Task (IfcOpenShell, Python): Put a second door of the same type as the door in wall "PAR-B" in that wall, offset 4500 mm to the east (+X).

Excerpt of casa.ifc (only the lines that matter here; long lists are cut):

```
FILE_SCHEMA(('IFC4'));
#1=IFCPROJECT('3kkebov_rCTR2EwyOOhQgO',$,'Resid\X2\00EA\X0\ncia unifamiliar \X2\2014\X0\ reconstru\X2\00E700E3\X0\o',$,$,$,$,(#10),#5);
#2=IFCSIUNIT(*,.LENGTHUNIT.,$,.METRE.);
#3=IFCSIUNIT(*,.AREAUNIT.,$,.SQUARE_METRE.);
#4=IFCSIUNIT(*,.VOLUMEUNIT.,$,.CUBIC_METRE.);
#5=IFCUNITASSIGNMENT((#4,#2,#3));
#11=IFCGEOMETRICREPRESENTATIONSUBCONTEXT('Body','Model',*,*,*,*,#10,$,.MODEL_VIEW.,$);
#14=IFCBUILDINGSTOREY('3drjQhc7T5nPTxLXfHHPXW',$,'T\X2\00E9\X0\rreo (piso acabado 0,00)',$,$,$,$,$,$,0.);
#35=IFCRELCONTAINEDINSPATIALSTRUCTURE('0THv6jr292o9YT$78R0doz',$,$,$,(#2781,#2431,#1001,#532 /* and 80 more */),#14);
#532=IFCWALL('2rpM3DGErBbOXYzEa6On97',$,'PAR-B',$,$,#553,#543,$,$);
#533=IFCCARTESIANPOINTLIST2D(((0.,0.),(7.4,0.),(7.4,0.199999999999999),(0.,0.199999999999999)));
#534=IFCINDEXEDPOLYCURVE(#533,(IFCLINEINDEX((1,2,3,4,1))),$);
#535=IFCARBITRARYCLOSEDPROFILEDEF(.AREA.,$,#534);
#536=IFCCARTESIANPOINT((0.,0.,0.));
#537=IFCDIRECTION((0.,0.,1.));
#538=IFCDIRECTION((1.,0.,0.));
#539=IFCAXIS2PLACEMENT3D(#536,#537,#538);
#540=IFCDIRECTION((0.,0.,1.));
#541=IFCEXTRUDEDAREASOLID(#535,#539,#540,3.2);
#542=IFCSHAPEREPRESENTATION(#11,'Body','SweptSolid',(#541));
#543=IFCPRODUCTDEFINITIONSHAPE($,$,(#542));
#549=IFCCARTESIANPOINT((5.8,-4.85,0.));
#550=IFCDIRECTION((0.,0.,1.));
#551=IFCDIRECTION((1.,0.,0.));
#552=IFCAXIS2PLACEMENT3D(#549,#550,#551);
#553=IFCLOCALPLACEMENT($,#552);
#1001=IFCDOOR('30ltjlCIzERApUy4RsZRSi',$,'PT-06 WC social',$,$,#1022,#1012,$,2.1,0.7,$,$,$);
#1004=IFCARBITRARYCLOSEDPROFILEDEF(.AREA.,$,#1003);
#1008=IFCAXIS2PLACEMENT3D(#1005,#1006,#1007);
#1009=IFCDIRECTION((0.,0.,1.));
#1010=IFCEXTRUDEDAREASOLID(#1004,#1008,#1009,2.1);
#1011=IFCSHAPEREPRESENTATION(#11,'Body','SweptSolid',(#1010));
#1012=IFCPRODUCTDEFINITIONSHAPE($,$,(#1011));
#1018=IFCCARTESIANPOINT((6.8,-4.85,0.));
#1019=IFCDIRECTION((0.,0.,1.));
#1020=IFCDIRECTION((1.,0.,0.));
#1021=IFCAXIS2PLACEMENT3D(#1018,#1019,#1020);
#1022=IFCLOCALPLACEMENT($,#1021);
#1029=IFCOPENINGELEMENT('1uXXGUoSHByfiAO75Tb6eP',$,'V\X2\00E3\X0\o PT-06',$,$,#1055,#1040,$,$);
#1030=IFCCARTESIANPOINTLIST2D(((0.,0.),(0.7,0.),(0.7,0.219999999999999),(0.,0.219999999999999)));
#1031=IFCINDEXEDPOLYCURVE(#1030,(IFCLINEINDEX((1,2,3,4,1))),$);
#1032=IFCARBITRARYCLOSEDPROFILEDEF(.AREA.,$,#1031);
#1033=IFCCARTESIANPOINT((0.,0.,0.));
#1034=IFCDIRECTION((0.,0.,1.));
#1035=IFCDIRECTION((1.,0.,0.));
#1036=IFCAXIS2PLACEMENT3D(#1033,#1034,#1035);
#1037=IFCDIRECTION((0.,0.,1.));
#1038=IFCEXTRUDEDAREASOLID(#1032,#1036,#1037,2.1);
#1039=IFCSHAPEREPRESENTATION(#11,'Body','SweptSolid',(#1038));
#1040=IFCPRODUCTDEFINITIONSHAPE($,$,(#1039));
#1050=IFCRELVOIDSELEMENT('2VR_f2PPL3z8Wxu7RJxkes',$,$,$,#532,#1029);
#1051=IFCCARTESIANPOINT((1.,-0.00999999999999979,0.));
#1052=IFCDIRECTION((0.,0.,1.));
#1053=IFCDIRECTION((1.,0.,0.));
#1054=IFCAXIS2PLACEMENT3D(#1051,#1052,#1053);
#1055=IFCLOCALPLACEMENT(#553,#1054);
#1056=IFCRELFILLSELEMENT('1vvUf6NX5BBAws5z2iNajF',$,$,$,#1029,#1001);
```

```python
import ifcopenshell
import ifcopenshell.api.feature
import ifcopenshell.api.geometry
import ifcopenshell.api.root
import ifcopenshell.geom
import ifcopenshell.util.element
import ifcopenshell.util.placement
import ifcopenshell.util.shape
import ifcopenshell.util.unit

model = ifcopenshell.open("casa.ifc")
unit_scale = ifcopenshell.util.unit.calculate_unit_scale(model)
settings = ifcopenshell.geom.settings()


def volume(element):
    """Net volume in cubic metres, openings subtracted."""
    shape = ifcopenshell.geom.create_shape(settings, element)
    return ifcopenshell.util.shape.get_volume(shape.geometry)


door = model.by_guid("30ltjlCIzERApUy4RsZRSi")
opening = door.FillsVoids[0].RelatingOpeningElement
wall = opening.VoidsElements[0].RelatingBuildingElement
before = volume(wall)
shift = ifcopenshell.util.placement.get_local_placement(wall.ObjectPlacement)[:3, 0] * 4.5 / unit_scale

# copy_class copies the void relationship, type, container and properties, but no geometry.
new_opening = ifcopenshell.api.root.copy_class(model, product=opening)
new_opening.Representation = ifcopenshell.util.element.copy_deep(
    model, opening.Representation, exclude=["IfcGeometricRepresentationContext", "IfcRepresentationMap"]
)
new_door = ifcopenshell.api.root.copy_class(model, product=door)
new_door.Representation = ifcopenshell.util.element.copy_deep(
    model, door.Representation, exclude=["IfcGeometricRepresentationContext", "IfcRepresentationMap"]
)
ifcopenshell.api.feature.add_filling(model, opening=new_opening, element=new_door)

for old, new in ((opening, new_opening), (door, new_door)):
    matrix = ifcopenshell.util.placement.get_local_placement(old.ObjectPlacement)
    matrix[:3, 3] += shift
    ifcopenshell.api.geometry.edit_object_placement(model, product=new, matrix=matrix, is_si=False)

after = volume(wall)

print(f"wall volume {before:.3f} -> {after:.3f} m3")

model.write("casa_updated.ifc")
```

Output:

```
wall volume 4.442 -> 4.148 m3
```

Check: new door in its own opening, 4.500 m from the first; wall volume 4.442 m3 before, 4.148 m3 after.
